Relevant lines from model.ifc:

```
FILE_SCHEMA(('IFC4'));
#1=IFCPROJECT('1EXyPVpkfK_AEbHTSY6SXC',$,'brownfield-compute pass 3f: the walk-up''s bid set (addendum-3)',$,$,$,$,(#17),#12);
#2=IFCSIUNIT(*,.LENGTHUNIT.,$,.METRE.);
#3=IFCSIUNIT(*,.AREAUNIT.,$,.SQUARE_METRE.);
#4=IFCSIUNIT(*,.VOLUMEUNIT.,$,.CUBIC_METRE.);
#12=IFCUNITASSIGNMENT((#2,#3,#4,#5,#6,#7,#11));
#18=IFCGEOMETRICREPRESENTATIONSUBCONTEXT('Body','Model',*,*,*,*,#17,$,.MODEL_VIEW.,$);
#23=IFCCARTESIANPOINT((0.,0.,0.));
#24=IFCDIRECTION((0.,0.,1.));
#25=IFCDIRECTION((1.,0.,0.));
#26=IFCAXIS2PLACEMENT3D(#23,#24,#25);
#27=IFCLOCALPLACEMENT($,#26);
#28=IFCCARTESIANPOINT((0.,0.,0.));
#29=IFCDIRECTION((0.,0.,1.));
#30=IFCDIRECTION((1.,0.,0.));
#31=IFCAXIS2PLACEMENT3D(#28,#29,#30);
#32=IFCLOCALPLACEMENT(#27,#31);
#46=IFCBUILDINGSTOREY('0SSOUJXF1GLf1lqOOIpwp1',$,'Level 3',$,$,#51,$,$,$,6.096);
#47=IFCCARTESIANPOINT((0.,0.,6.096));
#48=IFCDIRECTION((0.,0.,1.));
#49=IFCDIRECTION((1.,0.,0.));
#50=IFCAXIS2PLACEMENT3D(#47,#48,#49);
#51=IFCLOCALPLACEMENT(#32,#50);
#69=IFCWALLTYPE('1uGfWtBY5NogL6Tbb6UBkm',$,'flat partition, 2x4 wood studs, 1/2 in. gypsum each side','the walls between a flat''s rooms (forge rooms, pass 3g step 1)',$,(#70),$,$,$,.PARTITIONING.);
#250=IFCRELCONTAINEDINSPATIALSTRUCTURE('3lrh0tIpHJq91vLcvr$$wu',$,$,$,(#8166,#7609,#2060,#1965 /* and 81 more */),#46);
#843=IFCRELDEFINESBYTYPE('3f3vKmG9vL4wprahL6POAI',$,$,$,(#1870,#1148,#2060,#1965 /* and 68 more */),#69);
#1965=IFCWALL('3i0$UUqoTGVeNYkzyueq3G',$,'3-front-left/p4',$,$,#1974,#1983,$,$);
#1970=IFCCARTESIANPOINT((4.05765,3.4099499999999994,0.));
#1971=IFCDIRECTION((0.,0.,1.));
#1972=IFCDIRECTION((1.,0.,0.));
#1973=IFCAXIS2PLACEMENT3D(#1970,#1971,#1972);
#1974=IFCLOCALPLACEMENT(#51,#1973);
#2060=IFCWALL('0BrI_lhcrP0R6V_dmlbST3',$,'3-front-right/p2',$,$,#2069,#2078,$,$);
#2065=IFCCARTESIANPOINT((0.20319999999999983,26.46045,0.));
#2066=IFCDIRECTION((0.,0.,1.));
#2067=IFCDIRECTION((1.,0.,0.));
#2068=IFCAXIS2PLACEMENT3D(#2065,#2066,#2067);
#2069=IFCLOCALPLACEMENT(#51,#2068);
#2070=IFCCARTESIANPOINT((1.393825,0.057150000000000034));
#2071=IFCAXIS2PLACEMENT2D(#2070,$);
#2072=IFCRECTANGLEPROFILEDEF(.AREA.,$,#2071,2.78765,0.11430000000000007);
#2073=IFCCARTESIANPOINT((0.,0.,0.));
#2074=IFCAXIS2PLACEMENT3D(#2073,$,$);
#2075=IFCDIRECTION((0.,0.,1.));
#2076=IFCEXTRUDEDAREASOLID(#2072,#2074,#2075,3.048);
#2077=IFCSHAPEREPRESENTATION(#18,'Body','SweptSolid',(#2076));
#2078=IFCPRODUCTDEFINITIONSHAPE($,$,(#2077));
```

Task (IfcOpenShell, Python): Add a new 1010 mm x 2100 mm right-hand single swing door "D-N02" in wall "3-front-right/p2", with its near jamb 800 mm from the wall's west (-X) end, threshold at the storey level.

```python
import numpy as np
import ifcopenshell
import ifcopenshell.api.feature
import ifcopenshell.api.geometry
import ifcopenshell.api.root
import ifcopenshell.api.spatial
import ifcopenshell.geom
import ifcopenshell.util.element
import ifcopenshell.util.placement
import ifcopenshell.util.representation
import ifcopenshell.util.shape
import ifcopenshell.util.unit

model = ifcopenshell.open("model.ifc")
unit_scale = ifcopenshell.util.unit.calculate_unit_scale(model)
settings = ifcopenshell.geom.settings()


def volume(element):
    """Net volume in cubic metres, openings subtracted."""
    shape = ifcopenshell.geom.create_shape(settings, element)
    return ifcopenshell.util.shape.get_volume(shape.geometry)


wall = model.by_id(2060)
storey = ifcopenshell.util.element.get_container(wall, ifc_class="IfcBuildingStorey")
context = ifcopenshell.util.representation.get_context(model, "Model", "Body", "MODEL_VIEW")
before = volume(wall)

width, height, from_end, sill = 1.01, 2.1, 0.8, 0.0  # metres

# The wall runs along its own X axis, and the end named is its -X end.
wall_shape = ifcopenshell.geom.create_shape(settings, wall)
x, y, z = ifcopenshell.util.shape.get_vertices(wall_shape.geometry).T
start = x.min() + from_end
face, thickness = float(y.min()), float(y.max() - y.min())
wall_matrix = ifcopenshell.util.placement.get_local_placement(wall.ObjectPlacement)
level = ifcopenshell.util.placement.get_local_placement(storey.ObjectPlacement)[2, 3]


def in_wall(x, y):
    """Placement at x, y metres in the wall's axes, at sill height."""
    matrix = wall_matrix.copy()
    matrix[:, 3] = wall_matrix @ np.array([x / unit_scale, y / unit_scale, 0.0, 1.0])
    matrix[2, 3] = level + sill / unit_scale
    return matrix


# Opening: a box that overshoots both wall faces by 50 mm.
opening = ifcopenshell.api.root.create_entity(model, ifc_class="IfcOpeningElement", predefined_type="OPENING")
box = ifcopenshell.api.geometry.add_wall_representation(
    model, context=context, length=width, height=height, thickness=thickness + 0.1
)
ifcopenshell.api.geometry.assign_representation(model, product=opening, representation=box)
ifcopenshell.api.geometry.edit_object_placement(model, product=opening, matrix=in_wall(start, face - 0.05), is_si=False)
ifcopenshell.api.feature.add_feature(model, feature=opening, element=wall)

door = ifcopenshell.api.root.create_entity(model, ifc_class="IfcDoor", name="D-N02", predefined_type="DOOR")
door.OverallWidth, door.OverallHeight = width / unit_scale, height / unit_scale
door.OperationType = "SINGLE_SWING_RIGHT"
body = ifcopenshell.api.geometry.add_door_representation(
    model,
    context=context,
    overall_width=door.OverallWidth,
    overall_height=door.OverallHeight,
    operation_type="SINGLE_SWING_RIGHT",
    lining_properties={"LiningDepth": thickness / unit_scale, "ThresholdDepth": thickness / unit_scale},
)
ifcopenshell.api.geometry.assign_representation(model, product=door, representation=body)
ifcopenshell.api.spatial.assign_container(model, products=[door], relating_structure=storey)
ifcopenshell.api.feature.add_filling(model, opening=opening, element=door)

# The lining spans the wall, so the door starts at the wall face.
ifcopenshell.api.geometry.edit_object_placement(model, product=door, matrix=in_wall(start, face), is_si=False)

after = volume(wall)

print(f"wall volume {before:.3f} -> {after:.3f} m3")

model.write("model_updated.ifc")
```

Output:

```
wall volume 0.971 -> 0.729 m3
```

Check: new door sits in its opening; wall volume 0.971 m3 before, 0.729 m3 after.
